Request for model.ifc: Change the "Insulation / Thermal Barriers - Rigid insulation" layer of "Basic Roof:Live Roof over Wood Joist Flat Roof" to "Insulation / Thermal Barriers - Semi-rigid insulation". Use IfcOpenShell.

First a look at what the model holds.

```python
import ifcopenshell
import ifcopenshell.util.element

model = ifcopenshell.open("model.ifc")
print(model.schema)
for layer_set in model.by_type("IfcMaterialLayerSet"):
    if layer_set.LayerSetName == "Basic Roof:Live Roof over Wood Joist Flat Roof":
        for layer in layer_set.MaterialLayers:
            print(layer.id(), layer.Material and layer.Material.Name, layer.LayerThickness, sep=" | ")
        print(len(ifcopenshell.util.element.get_elements_by_material(model, layer_set)), "elements and types use it")
print(sorted(m.Name for m in model.by_type("IfcMaterial") if m.Name)[:60])
```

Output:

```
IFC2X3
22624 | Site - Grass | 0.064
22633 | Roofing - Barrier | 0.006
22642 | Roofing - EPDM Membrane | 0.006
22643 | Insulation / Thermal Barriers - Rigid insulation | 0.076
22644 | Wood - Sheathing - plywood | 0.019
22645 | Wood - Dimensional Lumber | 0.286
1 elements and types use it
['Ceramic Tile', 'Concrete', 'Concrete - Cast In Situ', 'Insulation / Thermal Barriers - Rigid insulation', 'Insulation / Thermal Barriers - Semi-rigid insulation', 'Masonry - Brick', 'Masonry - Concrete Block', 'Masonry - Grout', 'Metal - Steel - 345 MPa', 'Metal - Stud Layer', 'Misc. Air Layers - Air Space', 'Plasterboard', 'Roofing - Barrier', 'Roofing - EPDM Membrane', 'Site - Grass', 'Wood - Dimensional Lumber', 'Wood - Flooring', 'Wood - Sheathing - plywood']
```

```python
import ifcopenshell
import ifcopenshell.api.material

model = ifcopenshell.open("model.ifc")

layer_set = next(s for s in model.by_type("IfcMaterialLayerSet") if s.LayerSetName == "Basic Roof:Live Roof over Wood Joist Flat Roof")
layer = next(l for l in layer_set.MaterialLayers if l.Material and l.Material.Name == "Insulation / Thermal Barriers - Rigid insulation")
material = next(m for m in model.by_type("IfcMaterial") if m.Name == "Insulation / Thermal Barriers - Semi-rigid insulation")

# Point this one layer at the other material; renaming the old one would change it everywhere.
ifcopenshell.api.material.edit_layer(model, layer=layer, attributes={}, material=material)

print([l.Material.Name if l.Material else None for l in layer_set.MaterialLayers])

model.write("model_edited.ifc")
```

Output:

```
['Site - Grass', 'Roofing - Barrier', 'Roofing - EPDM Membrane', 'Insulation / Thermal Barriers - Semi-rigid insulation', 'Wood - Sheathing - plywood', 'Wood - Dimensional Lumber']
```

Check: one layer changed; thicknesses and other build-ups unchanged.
